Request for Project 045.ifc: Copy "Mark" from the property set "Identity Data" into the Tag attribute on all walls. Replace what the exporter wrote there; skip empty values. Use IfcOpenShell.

First a look at what the model holds.

```python
import ifcopenshell
import ifcopenshell.util.element

model = ifcopenshell.open("Project 045.ifc")
print(model.schema)
walls = model.by_type("IfcWall")
print(len(walls), "walls")
for e in walls[:8]:
    source = ifcopenshell.util.element.get_pset(e, "Identity Data", "Mark")
    target = e.Tag
    print(e.id(), repr(source), repr(target), sep=" | ")
```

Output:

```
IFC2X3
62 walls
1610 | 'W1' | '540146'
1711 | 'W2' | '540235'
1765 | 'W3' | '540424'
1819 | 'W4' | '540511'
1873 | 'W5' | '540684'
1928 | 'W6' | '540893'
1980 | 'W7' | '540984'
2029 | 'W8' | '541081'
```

```python
import ifcopenshell
import ifcopenshell.util.element

model = ifcopenshell.open("Project 045.ifc")

count = 0
for e in model.by_type("IfcWall"):
    value = ifcopenshell.util.element.get_pset(e, "Identity Data", "Mark")
    current = e.Tag
    if not value or not value.strip() or current == value:
        continue
    e.Tag = value
    count += 1

print(count, "walls updated")

model.write("Project 045_rev.ifc")
```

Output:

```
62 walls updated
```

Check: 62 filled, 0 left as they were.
